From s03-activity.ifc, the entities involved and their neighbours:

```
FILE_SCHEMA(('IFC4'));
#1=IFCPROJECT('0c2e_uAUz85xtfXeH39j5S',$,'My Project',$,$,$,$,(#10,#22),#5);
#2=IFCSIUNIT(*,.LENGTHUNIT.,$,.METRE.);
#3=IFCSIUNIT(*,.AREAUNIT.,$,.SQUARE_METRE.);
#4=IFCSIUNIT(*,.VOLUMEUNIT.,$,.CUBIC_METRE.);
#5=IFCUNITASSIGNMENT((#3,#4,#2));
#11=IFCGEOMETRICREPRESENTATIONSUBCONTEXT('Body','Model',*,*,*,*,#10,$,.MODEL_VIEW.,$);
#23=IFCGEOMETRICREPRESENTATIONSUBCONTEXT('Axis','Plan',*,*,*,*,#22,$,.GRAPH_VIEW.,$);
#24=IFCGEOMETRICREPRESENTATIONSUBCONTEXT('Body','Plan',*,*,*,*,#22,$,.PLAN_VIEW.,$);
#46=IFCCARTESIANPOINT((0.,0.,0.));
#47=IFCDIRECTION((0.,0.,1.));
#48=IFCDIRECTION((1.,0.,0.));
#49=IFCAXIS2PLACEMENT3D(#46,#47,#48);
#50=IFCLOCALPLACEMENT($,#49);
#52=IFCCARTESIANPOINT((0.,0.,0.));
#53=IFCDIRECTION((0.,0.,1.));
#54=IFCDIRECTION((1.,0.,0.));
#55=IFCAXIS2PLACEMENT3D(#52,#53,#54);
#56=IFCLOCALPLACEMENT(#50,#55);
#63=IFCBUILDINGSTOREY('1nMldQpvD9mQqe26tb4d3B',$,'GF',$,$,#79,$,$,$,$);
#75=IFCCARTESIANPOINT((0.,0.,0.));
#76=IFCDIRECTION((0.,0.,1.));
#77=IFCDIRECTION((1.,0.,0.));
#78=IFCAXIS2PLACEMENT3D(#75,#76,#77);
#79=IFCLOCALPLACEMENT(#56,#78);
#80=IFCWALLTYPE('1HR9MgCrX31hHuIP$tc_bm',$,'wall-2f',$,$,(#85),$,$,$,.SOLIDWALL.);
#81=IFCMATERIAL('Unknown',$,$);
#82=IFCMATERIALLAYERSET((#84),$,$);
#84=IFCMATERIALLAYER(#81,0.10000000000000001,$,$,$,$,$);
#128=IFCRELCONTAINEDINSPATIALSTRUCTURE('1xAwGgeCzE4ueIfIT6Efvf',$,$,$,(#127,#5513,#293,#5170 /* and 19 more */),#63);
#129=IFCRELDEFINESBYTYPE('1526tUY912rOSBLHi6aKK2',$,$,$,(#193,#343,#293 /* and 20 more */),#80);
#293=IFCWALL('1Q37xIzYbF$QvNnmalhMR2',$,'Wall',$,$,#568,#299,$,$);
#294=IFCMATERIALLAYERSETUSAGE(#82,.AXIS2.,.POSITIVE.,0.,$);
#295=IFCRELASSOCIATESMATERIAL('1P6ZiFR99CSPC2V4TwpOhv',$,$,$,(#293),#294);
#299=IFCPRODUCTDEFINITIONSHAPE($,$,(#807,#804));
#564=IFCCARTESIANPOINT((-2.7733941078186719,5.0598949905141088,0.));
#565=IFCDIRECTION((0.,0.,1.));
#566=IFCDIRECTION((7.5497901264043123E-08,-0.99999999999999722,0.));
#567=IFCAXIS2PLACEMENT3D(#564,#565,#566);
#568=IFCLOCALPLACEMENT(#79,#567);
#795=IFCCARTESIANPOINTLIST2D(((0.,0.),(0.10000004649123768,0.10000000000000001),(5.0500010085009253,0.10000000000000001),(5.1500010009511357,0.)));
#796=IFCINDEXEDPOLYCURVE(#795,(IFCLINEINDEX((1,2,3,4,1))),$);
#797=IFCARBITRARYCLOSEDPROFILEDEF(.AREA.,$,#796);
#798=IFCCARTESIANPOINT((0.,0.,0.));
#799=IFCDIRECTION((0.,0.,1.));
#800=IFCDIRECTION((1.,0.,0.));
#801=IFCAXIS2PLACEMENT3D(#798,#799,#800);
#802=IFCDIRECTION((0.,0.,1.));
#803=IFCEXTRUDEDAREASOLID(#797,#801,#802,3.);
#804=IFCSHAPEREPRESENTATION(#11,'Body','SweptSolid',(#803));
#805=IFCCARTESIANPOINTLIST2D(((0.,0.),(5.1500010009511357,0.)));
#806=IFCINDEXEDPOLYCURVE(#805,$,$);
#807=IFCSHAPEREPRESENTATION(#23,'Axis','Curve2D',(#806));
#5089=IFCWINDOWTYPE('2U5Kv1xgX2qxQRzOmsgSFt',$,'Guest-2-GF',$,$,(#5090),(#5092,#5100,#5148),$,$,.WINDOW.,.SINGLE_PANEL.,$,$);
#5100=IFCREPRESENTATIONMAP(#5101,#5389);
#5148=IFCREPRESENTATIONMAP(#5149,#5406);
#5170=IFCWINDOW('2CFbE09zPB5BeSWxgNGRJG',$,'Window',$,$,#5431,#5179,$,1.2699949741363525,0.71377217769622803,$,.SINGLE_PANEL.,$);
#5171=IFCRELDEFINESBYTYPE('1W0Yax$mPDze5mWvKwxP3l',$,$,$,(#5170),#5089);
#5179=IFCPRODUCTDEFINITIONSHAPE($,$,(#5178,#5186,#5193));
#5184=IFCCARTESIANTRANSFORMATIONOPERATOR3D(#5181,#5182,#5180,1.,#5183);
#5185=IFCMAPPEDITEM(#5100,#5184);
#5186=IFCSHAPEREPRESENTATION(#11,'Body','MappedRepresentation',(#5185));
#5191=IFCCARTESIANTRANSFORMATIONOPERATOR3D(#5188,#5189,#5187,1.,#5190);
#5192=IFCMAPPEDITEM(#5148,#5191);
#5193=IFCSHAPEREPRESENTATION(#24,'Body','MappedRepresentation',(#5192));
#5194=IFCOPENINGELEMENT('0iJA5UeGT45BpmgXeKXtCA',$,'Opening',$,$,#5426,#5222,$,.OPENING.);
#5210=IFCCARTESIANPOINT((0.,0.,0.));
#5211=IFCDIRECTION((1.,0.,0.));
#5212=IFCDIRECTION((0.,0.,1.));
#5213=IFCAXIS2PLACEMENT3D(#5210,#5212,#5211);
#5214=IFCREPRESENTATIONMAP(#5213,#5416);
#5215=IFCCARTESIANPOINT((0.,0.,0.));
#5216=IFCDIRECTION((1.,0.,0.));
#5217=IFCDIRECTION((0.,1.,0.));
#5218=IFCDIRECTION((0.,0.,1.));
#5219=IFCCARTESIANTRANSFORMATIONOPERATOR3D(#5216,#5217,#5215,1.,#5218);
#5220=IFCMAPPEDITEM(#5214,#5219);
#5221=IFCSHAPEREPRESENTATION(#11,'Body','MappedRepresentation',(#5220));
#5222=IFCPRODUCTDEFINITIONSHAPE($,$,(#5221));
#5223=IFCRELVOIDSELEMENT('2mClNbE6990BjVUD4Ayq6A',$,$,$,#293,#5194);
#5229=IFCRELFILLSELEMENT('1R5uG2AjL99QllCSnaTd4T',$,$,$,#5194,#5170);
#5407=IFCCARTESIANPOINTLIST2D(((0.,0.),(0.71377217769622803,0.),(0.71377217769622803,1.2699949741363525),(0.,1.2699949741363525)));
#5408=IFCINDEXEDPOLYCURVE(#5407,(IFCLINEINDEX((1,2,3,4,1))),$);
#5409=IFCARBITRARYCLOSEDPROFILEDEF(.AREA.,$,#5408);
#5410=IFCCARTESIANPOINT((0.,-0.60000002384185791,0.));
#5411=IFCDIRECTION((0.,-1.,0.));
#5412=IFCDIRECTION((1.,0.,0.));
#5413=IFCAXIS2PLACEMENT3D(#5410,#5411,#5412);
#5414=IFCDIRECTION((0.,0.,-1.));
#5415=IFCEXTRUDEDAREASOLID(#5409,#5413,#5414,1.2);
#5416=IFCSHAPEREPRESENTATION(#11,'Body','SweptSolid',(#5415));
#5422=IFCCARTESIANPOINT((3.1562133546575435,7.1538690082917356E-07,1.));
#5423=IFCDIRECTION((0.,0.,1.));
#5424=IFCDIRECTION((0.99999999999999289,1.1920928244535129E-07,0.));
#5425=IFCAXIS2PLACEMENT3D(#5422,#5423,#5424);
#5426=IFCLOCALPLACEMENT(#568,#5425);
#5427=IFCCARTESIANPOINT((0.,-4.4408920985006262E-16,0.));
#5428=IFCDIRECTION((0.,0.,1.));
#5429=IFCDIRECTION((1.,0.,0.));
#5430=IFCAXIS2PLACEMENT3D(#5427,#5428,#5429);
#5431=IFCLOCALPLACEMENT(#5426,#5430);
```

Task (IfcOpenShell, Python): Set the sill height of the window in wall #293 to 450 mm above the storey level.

```python
import numpy as np
import ifcopenshell
import ifcopenshell.api.geometry
import ifcopenshell.geom
import ifcopenshell.util.element
import ifcopenshell.util.placement
import ifcopenshell.util.shape
import ifcopenshell.util.unit

model = ifcopenshell.open("s03-activity.ifc")
unit_scale = ifcopenshell.util.unit.calculate_unit_scale(model)

window = model.by_guid("2CFbE09zPB5BeSWxgNGRJG")
opening = window.FillsVoids[0].RelatingOpeningElement
storey = ifcopenshell.util.element.get_container(window, ifc_class="IfcBuildingStorey")
level = ifcopenshell.util.placement.get_local_placement(storey.ObjectPlacement)[2, 3]

# The opening's origin need not be at the sill, so measure its lowest point.
shape = ifcopenshell.geom.create_shape(ifcopenshell.geom.settings(), opening)
bottom = ifcopenshell.util.shape.get_shape_bottom_elevation(shape, shape.geometry) / unit_scale
dz = level + 0.45 - bottom

shift = np.array([0.0, 0.0, dz])
# The window is placed relative to its opening, so it follows when the opening moves.
matrix = ifcopenshell.util.placement.get_local_placement(opening.ObjectPlacement)
matrix[:3, 3] += shift
ifcopenshell.api.geometry.edit_object_placement(
    model, product=opening, matrix=matrix, is_si=False, should_transform_children=True
)

print(f"moved by {dz * unit_scale:+.3f} m")

model.write("s03-activity_edited.ifc")
```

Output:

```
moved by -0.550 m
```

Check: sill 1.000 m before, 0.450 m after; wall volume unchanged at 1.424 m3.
